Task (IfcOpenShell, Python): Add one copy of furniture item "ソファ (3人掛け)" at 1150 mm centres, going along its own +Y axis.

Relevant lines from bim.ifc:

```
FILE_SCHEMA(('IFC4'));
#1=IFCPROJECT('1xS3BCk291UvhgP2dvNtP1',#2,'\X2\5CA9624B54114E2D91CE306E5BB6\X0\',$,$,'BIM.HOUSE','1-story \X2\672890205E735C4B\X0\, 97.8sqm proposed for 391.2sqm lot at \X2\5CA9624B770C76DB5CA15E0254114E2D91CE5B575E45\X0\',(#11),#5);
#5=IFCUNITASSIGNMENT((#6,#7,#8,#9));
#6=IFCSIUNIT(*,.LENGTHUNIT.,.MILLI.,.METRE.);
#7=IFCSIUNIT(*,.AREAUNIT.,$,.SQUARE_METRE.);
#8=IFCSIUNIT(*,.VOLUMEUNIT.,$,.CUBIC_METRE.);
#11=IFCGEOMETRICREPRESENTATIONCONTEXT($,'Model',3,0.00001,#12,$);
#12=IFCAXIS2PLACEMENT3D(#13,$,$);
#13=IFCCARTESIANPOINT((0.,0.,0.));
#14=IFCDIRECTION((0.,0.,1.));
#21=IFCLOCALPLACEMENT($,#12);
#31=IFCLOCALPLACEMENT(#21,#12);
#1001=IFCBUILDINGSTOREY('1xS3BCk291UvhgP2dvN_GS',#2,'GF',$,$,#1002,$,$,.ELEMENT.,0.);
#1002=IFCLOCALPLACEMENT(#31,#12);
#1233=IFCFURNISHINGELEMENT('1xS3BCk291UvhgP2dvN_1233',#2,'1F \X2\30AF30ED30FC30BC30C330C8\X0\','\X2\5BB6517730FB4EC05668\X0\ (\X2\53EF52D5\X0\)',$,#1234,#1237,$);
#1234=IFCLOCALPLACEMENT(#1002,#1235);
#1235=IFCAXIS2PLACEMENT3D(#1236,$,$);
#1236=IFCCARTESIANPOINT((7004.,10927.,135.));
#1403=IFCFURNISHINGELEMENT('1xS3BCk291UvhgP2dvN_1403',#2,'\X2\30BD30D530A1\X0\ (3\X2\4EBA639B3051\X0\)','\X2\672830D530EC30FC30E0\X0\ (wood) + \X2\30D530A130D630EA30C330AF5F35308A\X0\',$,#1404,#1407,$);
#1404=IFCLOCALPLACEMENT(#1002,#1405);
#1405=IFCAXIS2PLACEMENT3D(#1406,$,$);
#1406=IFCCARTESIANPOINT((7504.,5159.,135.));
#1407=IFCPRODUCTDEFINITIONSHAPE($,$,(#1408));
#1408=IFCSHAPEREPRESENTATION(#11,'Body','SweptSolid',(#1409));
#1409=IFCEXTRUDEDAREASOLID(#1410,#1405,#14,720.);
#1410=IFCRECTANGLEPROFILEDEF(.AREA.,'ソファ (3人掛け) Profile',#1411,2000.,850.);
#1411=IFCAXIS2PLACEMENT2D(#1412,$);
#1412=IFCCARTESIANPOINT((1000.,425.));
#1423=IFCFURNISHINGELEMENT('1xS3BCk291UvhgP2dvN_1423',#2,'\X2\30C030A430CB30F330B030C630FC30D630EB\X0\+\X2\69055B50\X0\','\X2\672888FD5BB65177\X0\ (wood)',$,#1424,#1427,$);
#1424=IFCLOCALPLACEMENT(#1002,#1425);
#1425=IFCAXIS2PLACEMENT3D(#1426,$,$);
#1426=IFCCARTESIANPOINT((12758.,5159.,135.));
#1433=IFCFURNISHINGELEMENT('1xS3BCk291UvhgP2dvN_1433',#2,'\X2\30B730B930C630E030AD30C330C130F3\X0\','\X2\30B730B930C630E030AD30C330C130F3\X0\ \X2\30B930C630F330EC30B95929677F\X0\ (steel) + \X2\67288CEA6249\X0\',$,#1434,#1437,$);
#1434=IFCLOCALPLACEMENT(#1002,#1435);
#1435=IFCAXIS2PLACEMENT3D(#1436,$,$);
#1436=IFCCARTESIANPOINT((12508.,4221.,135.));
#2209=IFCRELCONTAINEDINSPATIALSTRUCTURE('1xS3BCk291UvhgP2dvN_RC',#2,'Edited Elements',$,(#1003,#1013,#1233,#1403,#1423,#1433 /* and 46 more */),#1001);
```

```python
import ifcopenshell
import ifcopenshell.api.geometry
import ifcopenshell.api.root
import ifcopenshell.util.element
import ifcopenshell.util.placement

model = ifcopenshell.open("bim.ifc")


def reuse_history(source, copy):
    """copy_class also copies each property set's owner history, people and application; keep the originals."""
    for rel in copy.IsDefinedBy:
        if rel.is_a("IfcRelDefinesByProperties") and (history := rel.RelatingPropertyDefinition.OwnerHistory):
            rel.RelatingPropertyDefinition.OwnerHistory = source.OwnerHistory
            ifcopenshell.util.element.remove_deep2(model, history)


source = model.by_id(1403)
base = ifcopenshell.util.placement.get_local_placement(source.ObjectPlacement)
step = base[:3, 1] * 1150.0

for i in range(1, 2):
    copy = ifcopenshell.api.root.copy_class(model, product=source)
    copy.Representation = ifcopenshell.util.element.copy_deep(
        model, source.Representation, exclude=["IfcGeometricRepresentationContext", "IfcRepresentationMap"]
    )
    reuse_history(source, copy)
    matrix = base.copy()
    matrix[:3, 3] += i * step
    print("added at", matrix[:3, 3].round(3) + 0.0)
    ifcopenshell.api.geometry.edit_object_placement(model, product=copy, matrix=matrix, is_si=False)

model.write("bim_rev.ifc")
```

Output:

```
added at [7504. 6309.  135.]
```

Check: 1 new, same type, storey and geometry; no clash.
